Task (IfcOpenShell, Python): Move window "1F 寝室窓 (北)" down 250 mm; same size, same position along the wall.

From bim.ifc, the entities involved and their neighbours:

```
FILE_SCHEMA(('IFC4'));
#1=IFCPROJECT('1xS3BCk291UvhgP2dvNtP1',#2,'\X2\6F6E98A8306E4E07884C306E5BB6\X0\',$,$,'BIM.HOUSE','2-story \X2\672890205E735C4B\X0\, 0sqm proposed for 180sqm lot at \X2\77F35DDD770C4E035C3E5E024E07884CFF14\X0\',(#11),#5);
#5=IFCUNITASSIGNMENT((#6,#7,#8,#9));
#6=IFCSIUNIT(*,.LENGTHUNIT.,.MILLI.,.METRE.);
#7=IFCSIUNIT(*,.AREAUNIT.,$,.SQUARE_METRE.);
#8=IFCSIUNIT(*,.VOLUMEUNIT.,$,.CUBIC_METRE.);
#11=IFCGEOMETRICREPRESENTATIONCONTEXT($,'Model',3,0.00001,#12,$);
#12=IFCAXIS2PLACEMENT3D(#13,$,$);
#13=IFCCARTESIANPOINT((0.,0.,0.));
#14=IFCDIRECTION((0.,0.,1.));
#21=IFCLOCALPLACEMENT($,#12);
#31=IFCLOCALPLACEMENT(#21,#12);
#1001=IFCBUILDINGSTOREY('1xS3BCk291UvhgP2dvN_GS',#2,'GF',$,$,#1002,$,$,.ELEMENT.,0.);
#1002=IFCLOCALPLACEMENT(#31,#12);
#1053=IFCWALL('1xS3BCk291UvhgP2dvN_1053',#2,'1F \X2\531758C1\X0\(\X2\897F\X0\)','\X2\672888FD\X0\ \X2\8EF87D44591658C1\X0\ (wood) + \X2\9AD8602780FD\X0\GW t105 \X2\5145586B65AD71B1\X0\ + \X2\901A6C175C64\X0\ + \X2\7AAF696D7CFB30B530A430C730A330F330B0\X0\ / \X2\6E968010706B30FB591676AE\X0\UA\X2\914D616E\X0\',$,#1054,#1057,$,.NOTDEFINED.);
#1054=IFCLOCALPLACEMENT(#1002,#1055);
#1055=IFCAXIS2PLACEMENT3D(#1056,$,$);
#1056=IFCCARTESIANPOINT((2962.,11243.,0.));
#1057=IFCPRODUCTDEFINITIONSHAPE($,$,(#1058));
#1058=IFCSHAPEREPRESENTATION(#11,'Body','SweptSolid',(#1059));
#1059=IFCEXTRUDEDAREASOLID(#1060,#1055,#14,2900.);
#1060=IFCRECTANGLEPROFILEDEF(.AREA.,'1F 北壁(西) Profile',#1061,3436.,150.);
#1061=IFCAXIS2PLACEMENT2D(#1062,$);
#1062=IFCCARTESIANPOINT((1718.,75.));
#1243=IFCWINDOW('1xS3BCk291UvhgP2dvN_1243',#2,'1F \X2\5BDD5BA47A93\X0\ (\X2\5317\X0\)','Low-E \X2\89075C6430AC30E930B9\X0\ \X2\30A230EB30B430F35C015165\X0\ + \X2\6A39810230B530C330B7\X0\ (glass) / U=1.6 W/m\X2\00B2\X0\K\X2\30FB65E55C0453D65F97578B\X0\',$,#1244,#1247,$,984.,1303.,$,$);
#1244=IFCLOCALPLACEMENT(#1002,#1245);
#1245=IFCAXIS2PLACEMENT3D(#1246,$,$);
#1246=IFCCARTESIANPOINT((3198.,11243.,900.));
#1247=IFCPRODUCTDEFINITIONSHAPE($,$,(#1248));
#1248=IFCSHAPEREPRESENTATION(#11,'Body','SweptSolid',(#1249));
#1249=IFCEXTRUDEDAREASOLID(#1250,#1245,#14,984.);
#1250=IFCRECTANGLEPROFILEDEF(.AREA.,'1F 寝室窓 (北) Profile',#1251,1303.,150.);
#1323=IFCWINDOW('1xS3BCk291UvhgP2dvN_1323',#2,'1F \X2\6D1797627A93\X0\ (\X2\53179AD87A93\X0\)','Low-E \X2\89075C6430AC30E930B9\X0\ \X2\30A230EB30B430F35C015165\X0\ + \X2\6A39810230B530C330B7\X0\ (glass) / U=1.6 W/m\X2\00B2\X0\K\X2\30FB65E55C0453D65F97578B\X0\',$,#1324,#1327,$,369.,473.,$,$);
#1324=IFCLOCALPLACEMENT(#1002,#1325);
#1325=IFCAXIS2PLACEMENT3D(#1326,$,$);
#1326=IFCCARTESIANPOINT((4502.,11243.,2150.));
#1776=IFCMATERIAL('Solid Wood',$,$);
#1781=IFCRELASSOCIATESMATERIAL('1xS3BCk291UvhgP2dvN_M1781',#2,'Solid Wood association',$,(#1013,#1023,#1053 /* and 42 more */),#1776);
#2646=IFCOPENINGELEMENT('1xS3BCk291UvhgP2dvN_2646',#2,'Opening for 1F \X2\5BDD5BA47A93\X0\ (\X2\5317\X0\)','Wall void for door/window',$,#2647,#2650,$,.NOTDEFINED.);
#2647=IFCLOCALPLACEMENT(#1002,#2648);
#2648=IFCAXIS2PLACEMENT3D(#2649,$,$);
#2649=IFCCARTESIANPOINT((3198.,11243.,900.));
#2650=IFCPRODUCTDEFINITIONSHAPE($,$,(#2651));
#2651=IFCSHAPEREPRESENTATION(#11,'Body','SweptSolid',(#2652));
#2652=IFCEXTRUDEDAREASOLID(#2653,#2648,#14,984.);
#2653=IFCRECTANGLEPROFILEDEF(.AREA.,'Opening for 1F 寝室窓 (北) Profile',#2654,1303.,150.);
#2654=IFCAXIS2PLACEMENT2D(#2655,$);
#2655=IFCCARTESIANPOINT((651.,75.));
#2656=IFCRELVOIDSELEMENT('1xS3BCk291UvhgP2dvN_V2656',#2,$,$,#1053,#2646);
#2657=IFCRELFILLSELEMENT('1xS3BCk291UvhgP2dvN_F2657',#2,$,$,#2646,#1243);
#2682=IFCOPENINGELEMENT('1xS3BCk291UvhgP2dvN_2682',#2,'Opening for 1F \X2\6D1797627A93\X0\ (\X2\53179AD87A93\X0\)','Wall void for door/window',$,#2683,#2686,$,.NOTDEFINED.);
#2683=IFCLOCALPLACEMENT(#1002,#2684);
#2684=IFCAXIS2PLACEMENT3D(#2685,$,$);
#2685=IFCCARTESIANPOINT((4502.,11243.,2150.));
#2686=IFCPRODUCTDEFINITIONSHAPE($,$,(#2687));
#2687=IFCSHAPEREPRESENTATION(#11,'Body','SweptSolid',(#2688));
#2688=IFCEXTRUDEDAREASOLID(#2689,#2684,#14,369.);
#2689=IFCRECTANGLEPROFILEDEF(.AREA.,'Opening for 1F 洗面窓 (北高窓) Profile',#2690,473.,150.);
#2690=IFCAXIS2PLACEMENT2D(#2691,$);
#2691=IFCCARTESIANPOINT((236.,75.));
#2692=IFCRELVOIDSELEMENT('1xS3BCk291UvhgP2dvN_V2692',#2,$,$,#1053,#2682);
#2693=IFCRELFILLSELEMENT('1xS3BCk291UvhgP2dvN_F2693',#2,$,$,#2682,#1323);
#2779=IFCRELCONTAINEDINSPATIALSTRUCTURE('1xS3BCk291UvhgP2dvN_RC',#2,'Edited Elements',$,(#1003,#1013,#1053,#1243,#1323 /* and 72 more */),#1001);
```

```python
import numpy as np
import ifcopenshell
import ifcopenshell.api.geometry
import ifcopenshell.util.placement
import ifcopenshell.util.unit

model = ifcopenshell.open("bim.ifc")
unit_scale = ifcopenshell.util.unit.calculate_unit_scale(model)

window = model.by_id(1243)
opening = window.FillsVoids[0].RelatingOpeningElement
dz = -0.25 / unit_scale

shift = np.array([0.0, 0.0, dz])
# The window is not placed relative to its opening, so move both.
for product in (opening, window):
    matrix = ifcopenshell.util.placement.get_local_placement(product.ObjectPlacement)
    matrix[:3, 3] += shift
    ifcopenshell.api.geometry.edit_object_placement(model, product=product, matrix=matrix, is_si=False)

print(f"moved by {dz * unit_scale:+.3f} m")

model.write("bim_v2.ifc")
```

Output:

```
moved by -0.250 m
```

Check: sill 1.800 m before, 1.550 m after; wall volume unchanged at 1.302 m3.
